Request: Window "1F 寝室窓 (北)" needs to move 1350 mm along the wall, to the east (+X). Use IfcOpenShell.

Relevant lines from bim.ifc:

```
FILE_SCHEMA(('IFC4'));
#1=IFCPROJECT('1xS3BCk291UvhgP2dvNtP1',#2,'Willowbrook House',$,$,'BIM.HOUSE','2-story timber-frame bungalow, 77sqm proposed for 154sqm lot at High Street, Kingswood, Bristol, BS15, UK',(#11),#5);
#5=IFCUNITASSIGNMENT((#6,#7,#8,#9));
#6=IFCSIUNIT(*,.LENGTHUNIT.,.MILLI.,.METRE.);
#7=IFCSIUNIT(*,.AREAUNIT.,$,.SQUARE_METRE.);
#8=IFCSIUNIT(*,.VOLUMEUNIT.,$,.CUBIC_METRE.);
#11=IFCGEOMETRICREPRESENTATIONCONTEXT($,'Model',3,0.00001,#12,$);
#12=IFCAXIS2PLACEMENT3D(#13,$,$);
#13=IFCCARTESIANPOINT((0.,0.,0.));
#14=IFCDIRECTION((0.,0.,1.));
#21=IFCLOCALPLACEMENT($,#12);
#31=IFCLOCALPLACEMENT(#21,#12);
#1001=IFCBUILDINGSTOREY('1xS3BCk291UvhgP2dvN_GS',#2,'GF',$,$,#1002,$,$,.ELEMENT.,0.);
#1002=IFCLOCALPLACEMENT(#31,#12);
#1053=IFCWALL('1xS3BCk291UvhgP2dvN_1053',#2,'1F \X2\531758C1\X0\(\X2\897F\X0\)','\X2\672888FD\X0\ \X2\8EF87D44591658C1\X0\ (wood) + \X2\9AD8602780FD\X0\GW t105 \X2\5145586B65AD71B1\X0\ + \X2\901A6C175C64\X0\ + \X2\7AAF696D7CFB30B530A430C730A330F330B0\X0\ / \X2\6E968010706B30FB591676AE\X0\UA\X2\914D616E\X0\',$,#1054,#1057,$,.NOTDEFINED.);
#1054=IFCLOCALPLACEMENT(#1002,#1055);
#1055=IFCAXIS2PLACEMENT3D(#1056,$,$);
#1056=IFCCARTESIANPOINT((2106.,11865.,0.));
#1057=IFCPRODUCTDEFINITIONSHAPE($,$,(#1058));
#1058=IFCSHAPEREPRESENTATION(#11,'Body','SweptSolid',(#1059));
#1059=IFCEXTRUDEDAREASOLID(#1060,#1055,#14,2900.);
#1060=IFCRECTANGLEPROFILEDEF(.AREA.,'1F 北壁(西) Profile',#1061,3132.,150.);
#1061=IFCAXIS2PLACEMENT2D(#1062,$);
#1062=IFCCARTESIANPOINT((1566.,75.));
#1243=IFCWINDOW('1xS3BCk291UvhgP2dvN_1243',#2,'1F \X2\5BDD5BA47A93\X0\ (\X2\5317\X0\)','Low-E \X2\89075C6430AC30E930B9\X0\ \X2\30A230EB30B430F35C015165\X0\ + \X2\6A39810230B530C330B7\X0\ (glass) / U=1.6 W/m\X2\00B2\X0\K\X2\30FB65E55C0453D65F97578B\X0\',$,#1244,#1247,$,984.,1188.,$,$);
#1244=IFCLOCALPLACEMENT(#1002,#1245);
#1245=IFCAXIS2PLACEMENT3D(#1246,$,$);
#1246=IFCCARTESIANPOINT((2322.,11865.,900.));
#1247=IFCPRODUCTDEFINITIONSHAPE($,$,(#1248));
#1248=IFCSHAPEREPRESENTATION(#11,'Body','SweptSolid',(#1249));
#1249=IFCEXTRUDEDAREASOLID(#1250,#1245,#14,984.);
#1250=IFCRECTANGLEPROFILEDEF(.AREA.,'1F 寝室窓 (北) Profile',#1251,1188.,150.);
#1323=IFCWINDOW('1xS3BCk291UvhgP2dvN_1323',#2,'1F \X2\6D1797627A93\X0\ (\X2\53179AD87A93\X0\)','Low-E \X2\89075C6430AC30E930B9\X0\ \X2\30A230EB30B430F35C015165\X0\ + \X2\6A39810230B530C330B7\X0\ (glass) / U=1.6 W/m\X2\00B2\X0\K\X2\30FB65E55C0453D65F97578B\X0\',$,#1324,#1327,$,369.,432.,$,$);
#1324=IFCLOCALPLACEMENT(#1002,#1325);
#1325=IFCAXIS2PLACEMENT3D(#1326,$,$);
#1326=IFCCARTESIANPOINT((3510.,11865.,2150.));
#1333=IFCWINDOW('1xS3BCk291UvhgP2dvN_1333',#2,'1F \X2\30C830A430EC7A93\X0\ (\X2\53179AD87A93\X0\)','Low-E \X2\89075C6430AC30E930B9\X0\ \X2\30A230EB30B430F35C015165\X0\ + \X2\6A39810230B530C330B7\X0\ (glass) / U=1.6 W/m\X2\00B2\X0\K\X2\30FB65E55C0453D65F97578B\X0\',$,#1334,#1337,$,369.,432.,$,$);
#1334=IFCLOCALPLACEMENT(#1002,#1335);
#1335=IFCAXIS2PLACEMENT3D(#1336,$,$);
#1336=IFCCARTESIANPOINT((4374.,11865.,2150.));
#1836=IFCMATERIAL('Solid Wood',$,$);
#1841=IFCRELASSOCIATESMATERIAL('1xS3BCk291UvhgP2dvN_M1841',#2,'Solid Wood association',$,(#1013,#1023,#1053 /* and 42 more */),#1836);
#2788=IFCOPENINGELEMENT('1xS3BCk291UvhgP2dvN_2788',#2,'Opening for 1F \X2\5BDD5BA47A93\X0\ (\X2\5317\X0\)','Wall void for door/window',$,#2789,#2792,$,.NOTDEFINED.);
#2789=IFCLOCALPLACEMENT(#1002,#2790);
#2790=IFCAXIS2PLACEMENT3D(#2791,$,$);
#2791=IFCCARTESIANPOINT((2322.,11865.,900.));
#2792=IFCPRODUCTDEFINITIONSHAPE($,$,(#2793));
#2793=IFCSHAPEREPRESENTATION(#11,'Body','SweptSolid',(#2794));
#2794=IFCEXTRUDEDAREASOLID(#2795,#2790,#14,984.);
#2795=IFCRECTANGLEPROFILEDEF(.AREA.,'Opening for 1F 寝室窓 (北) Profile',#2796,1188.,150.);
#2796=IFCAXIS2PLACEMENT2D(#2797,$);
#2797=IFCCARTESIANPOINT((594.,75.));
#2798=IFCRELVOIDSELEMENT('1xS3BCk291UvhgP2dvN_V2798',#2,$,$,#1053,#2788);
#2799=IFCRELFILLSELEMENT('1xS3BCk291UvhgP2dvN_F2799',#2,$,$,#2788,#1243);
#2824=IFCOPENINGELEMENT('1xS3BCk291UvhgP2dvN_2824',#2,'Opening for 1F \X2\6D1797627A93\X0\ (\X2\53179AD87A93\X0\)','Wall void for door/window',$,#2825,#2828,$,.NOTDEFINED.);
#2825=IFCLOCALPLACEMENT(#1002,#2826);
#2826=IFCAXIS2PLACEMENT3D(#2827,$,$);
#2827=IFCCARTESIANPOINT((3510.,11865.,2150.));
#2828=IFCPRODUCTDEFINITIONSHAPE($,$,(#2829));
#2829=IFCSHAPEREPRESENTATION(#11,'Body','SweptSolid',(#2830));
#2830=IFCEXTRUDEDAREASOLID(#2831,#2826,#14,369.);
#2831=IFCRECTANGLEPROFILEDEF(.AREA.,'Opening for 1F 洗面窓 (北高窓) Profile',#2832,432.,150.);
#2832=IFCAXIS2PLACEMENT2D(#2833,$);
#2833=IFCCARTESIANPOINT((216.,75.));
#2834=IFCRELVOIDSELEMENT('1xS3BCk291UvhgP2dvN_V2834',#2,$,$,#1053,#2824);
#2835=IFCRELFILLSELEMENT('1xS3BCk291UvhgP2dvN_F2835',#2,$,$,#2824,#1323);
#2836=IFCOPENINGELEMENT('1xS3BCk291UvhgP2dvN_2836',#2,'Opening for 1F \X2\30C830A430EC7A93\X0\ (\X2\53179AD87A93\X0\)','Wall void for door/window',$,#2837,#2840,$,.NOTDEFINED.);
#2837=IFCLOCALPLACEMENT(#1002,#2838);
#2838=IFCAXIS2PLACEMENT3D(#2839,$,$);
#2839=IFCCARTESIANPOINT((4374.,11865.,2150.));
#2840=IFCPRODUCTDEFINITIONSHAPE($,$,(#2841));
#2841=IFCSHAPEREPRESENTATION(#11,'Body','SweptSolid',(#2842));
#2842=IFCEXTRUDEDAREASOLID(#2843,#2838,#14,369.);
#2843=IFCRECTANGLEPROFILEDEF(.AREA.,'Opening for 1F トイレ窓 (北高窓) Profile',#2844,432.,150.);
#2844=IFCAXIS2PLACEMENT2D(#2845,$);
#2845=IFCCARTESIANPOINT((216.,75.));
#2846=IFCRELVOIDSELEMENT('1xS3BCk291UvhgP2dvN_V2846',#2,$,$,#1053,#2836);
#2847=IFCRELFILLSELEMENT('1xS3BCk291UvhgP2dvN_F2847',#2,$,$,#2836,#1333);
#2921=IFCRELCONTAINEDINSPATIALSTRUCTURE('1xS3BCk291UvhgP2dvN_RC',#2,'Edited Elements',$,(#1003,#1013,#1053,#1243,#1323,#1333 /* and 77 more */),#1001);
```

```python
import ifcopenshell
import ifcopenshell.api.geometry
import ifcopenshell.util.placement

model = ifcopenshell.open("bim.ifc")

window = model.by_guid("1xS3BCk291UvhgP2dvN_1243")
opening = window.FillsVoids[0].RelatingOpeningElement
wall = opening.VoidsElements[0].RelatingBuildingElement

wall_matrix = ifcopenshell.util.placement.get_local_placement(wall.ObjectPlacement)
shift = wall_matrix[:3, 0] * 1350.0
before = ifcopenshell.util.placement.get_local_placement(window.ObjectPlacement)[:3, 3].copy()

# The window is not placed relative to its opening, so move both.
for product in (opening, window):
    matrix = ifcopenshell.util.placement.get_local_placement(product.ObjectPlacement)
    matrix[:3, 3] += shift
    ifcopenshell.api.geometry.edit_object_placement(model, product=product, matrix=matrix, is_si=False)

after = ifcopenshell.util.placement.get_local_placement(window.ObjectPlacement)[:3, 3]
print("window moved by", (after - before).round(3) + 0.0)

model.write("bim-out.ifc")
```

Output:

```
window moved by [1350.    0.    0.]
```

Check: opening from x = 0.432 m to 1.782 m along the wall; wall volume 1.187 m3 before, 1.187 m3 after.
